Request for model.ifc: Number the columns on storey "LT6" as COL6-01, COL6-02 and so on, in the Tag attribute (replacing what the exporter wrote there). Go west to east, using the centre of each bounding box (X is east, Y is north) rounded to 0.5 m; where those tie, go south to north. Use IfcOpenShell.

First a look at what the model holds.

```python
import ifcopenshell
import ifcopenshell.util.element
import ifcopenshell.util.placement

model = ifcopenshell.open("model.ifc")
print(model.schema)
storey = next(s for s in model.by_type("IfcBuildingStorey") if s.Name == "LT6")
columns = [e for e in ifcopenshell.util.element.get_decomposition(storey) if e.is_a("IfcColumn")]
for e in sorted(columns, key=lambda e: e.id()):
    origin = ifcopenshell.util.placement.get_local_placement(e.ObjectPlacement)[:3, 3]
    print(e.id(), e.Tag, e.Name, origin.round(2) + 0.0, sep=" | ")
```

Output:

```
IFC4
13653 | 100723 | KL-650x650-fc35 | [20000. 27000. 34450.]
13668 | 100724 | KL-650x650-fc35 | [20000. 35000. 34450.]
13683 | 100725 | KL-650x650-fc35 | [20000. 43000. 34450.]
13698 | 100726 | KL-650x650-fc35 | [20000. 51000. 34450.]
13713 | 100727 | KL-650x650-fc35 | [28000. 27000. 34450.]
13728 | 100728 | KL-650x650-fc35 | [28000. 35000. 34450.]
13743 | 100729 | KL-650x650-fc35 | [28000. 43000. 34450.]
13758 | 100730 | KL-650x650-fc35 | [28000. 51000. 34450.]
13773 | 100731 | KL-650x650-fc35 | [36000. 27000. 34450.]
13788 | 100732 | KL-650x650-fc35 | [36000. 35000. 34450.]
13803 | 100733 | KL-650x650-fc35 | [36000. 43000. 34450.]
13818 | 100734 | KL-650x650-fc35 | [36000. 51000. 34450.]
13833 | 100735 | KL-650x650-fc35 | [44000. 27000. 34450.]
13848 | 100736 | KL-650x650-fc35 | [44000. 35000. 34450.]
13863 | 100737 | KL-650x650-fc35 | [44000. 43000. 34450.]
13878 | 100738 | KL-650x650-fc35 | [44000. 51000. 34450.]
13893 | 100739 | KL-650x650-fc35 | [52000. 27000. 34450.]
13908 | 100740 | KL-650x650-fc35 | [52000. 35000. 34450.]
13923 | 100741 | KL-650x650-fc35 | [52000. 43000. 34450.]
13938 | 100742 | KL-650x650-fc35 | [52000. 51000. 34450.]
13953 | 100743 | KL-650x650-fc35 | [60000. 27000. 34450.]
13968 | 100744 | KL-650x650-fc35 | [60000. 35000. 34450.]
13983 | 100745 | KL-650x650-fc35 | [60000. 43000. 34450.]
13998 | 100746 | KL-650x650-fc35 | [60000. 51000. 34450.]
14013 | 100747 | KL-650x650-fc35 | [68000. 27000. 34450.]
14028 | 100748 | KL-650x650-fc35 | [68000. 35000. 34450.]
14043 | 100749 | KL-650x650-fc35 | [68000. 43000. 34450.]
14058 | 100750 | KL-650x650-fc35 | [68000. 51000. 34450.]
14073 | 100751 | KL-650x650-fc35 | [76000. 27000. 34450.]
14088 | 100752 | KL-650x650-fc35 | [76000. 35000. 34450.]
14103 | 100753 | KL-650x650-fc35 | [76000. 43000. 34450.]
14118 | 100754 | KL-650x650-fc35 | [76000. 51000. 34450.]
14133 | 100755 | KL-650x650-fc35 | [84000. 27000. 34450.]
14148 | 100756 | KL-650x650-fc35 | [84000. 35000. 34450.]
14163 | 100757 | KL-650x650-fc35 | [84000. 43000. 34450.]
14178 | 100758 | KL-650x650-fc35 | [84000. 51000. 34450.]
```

```python
import ifcopenshell
import ifcopenshell.geom
import ifcopenshell.util.element
import ifcopenshell.util.shape

model = ifcopenshell.open("model.ifc")
settings = ifcopenshell.geom.settings()
settings.set("use-world-coords", True)


def centre(element):
    shape = ifcopenshell.geom.create_shape(settings, element)
    return ifcopenshell.util.shape.get_bbox_centroid(shape.geometry)


storey = next(s for s in model.by_type("IfcBuildingStorey") if s.Name == "LT6")
columns = [e for e in ifcopenshell.util.element.get_decomposition(storey) if e.is_a("IfcColumn")]

# Insertion points can sit at a corner or the storey origin, so sort by the geometry (in metres).
centres = {e: centre(e) for e in columns}
columns.sort(key=lambda e: (round(centres[e][0] / 0.5), centres[e][1]))

for i, e in enumerate(columns, start=1):
    number = f"COL6-{i:02d}"
    e.Tag = number
    print(e.id(), number)

model.write("model_rev.ifc")
```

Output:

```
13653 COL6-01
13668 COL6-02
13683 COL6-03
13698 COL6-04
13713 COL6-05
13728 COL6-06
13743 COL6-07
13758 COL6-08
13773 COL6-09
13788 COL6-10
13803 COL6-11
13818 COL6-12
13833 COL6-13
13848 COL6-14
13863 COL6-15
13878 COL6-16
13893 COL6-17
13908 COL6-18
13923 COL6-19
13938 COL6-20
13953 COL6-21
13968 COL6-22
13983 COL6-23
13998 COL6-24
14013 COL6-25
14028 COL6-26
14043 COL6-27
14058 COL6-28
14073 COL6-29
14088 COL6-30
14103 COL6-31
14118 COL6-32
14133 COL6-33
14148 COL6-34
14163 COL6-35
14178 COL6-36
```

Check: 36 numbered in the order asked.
